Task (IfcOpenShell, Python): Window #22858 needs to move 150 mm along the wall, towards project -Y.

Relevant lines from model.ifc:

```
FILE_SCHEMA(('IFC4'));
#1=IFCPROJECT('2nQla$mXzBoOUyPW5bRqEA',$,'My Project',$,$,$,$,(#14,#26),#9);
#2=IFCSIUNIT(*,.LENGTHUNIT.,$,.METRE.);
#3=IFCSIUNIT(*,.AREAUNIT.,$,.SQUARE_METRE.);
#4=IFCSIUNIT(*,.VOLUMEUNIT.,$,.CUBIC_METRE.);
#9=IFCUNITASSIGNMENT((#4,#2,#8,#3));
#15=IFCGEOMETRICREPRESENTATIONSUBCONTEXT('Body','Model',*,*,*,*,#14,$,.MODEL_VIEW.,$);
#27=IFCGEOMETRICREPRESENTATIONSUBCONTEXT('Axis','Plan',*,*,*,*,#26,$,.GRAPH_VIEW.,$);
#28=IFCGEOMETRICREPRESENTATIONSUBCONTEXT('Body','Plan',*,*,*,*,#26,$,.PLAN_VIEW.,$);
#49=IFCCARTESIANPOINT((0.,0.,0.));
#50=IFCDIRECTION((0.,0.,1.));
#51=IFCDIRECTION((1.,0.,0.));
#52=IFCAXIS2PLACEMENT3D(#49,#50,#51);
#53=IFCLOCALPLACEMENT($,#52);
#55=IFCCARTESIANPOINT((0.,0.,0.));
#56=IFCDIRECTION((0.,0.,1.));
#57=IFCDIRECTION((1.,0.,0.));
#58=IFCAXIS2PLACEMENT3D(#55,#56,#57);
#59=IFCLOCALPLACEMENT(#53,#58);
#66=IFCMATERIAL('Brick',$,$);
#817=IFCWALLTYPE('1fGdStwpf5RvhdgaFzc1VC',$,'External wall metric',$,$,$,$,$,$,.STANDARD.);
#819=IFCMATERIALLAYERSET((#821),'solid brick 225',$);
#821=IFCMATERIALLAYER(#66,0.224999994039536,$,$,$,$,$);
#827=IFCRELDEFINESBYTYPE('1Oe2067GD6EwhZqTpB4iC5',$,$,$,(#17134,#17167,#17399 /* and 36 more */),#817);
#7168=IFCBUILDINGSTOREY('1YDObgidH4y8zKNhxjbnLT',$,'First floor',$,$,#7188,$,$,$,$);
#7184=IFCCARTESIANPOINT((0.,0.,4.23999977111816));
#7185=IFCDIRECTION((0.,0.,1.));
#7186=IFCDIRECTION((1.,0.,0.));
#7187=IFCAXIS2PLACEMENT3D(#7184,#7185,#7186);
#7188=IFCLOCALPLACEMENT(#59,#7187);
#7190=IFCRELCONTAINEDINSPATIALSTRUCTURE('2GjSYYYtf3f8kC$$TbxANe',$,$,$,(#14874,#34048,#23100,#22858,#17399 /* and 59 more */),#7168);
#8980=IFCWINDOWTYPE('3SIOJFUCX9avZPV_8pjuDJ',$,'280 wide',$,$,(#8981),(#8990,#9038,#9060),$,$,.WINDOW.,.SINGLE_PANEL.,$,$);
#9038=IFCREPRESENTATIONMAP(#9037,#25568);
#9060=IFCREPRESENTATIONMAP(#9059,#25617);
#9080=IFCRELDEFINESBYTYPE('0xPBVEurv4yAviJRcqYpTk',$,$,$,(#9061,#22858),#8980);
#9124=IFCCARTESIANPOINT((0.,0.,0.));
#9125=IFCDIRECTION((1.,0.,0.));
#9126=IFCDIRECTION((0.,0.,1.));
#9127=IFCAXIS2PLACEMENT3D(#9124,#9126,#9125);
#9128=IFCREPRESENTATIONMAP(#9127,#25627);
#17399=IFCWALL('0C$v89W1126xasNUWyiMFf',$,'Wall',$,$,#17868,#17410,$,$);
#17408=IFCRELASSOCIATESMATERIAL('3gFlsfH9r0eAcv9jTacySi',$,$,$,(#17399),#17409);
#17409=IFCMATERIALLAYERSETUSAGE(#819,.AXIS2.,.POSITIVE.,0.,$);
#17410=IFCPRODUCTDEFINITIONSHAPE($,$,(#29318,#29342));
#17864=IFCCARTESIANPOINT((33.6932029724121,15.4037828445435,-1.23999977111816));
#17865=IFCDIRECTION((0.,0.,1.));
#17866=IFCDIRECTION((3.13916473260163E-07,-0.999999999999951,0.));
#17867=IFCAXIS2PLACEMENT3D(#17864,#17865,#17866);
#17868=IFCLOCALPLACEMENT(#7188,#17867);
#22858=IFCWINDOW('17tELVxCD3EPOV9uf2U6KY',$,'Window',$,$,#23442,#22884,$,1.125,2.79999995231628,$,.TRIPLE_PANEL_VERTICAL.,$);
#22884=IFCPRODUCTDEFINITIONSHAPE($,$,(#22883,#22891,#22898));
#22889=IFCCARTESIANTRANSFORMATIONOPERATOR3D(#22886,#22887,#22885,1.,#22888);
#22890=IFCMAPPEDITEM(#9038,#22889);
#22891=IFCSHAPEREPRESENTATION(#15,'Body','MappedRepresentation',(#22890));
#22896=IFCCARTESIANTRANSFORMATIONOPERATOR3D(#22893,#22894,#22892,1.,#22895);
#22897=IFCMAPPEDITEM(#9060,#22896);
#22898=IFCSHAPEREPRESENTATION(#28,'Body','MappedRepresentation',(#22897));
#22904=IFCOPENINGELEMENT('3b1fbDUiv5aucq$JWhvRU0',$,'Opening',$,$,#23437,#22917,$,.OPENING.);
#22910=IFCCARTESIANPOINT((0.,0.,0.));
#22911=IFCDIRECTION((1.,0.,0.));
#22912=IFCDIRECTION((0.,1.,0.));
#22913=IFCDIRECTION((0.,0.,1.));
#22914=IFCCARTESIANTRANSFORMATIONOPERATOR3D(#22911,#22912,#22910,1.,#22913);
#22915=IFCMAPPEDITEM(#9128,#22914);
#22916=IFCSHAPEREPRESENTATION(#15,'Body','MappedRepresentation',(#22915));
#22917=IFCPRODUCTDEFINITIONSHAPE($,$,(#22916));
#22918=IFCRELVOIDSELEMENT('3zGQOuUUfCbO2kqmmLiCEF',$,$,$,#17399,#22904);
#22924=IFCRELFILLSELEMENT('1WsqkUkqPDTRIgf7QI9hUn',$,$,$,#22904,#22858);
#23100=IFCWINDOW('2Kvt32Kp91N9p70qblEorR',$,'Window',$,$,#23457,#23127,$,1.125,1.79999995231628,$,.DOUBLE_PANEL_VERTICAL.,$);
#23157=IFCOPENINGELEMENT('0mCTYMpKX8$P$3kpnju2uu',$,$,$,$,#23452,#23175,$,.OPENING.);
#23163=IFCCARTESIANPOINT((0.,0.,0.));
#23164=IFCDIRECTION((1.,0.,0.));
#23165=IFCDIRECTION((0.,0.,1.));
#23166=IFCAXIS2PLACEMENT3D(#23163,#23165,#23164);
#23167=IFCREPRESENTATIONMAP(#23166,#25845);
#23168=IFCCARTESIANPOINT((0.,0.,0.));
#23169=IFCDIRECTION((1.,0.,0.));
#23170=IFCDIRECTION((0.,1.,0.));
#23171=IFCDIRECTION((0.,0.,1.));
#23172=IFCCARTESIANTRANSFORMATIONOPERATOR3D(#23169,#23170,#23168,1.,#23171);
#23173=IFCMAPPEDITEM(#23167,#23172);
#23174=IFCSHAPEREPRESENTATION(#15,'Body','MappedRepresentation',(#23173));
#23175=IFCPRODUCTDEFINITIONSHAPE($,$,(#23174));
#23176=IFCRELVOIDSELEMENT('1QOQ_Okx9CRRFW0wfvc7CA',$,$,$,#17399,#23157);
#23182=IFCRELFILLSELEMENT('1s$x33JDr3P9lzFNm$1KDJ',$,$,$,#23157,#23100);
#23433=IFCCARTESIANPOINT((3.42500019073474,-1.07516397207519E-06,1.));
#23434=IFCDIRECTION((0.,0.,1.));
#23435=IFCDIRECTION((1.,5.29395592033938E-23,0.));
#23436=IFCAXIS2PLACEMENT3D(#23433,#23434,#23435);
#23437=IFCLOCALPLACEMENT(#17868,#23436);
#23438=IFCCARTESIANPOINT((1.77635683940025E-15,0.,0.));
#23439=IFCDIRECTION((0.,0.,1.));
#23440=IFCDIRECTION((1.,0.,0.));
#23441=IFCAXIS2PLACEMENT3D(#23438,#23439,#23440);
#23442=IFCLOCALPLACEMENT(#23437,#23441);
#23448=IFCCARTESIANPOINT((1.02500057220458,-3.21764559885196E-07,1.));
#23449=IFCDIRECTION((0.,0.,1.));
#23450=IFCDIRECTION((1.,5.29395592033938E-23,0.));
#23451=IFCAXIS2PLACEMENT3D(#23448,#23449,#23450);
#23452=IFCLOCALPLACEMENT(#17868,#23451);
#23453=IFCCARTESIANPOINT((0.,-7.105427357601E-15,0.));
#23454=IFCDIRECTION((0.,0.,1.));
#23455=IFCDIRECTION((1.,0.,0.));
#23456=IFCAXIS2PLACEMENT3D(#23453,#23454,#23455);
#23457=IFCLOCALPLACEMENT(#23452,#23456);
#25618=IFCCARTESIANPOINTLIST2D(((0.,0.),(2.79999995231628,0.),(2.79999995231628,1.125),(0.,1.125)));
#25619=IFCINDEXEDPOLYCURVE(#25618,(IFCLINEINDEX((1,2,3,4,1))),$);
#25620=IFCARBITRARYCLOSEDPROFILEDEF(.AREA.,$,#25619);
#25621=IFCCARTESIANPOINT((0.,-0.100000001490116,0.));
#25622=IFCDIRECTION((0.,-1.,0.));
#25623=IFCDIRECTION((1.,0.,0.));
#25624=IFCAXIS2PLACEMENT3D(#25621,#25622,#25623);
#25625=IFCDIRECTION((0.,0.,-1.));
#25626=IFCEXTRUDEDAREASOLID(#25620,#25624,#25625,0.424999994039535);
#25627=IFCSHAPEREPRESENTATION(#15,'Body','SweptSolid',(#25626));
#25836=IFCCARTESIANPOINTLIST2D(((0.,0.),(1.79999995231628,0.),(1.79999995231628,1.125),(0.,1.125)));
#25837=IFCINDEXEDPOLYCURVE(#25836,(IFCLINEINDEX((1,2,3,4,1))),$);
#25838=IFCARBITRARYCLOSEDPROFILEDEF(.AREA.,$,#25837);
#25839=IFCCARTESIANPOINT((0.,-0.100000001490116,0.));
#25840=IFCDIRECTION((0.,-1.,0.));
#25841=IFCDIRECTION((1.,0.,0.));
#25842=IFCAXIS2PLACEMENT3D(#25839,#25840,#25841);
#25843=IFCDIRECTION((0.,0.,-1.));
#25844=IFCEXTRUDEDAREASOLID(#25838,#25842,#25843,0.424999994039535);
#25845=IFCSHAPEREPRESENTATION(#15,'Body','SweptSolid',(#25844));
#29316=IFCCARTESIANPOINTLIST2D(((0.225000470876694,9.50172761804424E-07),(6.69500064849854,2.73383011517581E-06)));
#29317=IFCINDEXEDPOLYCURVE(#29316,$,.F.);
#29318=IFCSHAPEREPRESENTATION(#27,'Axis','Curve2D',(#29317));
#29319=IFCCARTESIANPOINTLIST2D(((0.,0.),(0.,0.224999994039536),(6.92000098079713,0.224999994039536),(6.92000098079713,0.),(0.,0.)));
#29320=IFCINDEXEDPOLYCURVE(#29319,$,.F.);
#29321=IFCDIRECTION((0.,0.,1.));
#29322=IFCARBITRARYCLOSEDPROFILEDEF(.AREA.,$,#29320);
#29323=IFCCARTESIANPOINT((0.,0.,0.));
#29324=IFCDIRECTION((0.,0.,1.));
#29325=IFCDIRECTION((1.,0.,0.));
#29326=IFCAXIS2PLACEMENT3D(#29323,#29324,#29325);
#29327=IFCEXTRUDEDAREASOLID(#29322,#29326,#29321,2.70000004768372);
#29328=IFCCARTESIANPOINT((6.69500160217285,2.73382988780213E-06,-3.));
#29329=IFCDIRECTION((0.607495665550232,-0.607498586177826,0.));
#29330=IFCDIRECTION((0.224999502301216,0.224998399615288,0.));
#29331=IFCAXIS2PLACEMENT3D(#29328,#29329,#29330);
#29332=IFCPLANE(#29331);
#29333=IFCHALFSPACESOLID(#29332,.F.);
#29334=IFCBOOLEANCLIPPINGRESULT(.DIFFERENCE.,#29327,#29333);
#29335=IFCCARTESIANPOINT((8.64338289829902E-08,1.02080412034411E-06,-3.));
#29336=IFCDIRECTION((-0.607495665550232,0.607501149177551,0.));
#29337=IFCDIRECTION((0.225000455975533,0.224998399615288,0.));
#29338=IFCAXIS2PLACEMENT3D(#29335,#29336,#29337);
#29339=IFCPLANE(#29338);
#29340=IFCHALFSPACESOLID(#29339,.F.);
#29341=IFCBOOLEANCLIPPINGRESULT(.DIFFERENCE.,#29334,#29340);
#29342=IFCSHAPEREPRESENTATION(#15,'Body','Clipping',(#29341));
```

```python
import ifcopenshell
import ifcopenshell.api.geometry
import ifcopenshell.util.placement

model = ifcopenshell.open("model.ifc")

window = model.by_id(22858)
opening = window.FillsVoids[0].RelatingOpeningElement
wall = opening.VoidsElements[0].RelatingBuildingElement

wall_matrix = ifcopenshell.util.placement.get_local_placement(wall.ObjectPlacement)
shift = wall_matrix[:3, 0] * 0.15
before = ifcopenshell.util.placement.get_local_placement(window.ObjectPlacement)[:3, 3].copy()

# The window is placed relative to its opening, so it follows when the opening moves.
matrix = ifcopenshell.util.placement.get_local_placement(opening.ObjectPlacement)
matrix[:3, 3] += shift
ifcopenshell.api.geometry.edit_object_placement(
    model, product=opening, matrix=matrix, is_si=False, should_transform_children=True
)

after = ifcopenshell.util.placement.get_local_placement(window.ObjectPlacement)[:3, 3]
print("window moved by", (after - before).round(3) + 0.0)

model.write("model_v2.ifc")
```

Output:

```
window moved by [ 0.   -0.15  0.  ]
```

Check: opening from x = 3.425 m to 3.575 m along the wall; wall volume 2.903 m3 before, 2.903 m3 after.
